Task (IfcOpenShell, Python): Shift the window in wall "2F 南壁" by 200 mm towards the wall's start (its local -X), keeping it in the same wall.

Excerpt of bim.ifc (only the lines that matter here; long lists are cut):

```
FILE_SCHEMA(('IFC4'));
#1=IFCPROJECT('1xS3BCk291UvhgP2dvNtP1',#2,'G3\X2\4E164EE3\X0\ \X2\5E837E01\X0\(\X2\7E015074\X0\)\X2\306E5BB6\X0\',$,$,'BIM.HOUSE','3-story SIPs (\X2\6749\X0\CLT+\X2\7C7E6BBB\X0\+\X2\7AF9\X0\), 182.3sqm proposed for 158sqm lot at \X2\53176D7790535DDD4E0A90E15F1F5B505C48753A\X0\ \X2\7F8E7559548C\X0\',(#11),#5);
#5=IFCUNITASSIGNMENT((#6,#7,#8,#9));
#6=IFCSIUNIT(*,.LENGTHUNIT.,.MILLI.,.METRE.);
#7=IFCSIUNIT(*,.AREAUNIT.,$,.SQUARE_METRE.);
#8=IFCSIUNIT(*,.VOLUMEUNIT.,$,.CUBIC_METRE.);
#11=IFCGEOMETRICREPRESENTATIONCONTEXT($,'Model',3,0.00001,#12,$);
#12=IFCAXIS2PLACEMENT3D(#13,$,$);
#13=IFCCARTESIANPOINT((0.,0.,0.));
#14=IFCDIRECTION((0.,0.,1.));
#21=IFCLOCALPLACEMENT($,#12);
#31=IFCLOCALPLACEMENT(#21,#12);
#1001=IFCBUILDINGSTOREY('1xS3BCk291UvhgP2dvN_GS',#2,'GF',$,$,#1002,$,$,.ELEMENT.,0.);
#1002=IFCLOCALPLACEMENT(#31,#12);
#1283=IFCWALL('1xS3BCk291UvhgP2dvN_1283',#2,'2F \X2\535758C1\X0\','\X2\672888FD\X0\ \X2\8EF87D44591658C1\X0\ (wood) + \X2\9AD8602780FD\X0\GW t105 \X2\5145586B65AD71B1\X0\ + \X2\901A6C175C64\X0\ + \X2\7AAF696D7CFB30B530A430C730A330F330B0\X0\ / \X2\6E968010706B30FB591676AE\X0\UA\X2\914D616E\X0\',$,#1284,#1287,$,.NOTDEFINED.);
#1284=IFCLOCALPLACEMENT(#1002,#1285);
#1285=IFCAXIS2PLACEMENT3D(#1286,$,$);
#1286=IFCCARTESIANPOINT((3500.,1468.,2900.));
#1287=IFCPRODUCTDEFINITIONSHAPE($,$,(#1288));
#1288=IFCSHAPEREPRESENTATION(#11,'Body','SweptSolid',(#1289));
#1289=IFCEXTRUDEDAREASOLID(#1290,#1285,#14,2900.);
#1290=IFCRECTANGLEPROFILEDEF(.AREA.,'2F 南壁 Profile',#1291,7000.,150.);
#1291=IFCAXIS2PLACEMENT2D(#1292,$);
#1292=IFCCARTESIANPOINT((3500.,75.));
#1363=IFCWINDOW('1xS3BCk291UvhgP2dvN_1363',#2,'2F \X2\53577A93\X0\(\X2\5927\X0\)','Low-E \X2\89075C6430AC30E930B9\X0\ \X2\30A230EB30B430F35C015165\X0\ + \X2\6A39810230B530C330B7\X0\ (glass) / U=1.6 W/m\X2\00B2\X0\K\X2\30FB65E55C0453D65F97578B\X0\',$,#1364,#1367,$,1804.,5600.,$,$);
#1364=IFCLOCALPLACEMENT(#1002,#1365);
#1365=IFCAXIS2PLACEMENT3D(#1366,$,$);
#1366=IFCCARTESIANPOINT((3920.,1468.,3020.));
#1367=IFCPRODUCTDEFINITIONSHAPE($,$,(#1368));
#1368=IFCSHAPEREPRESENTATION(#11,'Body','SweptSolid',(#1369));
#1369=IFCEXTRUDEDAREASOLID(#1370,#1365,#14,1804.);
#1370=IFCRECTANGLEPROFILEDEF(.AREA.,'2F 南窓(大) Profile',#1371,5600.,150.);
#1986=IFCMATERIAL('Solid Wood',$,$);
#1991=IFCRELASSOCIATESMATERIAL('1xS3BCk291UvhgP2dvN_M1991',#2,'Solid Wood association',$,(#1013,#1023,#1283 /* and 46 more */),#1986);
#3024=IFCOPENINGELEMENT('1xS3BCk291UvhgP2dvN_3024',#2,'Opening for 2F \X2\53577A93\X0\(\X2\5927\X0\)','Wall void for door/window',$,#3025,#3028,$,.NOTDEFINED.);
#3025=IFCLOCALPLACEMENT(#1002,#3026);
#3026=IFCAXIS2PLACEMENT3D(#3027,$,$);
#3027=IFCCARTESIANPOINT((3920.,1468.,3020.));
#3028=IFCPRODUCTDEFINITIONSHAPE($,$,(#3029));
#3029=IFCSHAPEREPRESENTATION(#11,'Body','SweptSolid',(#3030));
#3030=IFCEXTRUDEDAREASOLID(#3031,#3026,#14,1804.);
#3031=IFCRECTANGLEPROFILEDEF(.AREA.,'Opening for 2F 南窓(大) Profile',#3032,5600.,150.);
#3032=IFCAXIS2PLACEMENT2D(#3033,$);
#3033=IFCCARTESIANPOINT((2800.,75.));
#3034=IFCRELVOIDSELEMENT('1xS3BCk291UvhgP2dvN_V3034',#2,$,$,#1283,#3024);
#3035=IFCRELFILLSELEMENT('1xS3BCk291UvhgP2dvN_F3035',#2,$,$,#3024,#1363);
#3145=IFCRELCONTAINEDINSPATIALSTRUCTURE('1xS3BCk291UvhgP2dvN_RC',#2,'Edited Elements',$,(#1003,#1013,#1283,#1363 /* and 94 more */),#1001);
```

```python
import ifcopenshell
import ifcopenshell.api.geometry
import ifcopenshell.util.placement
import ifcopenshell.util.unit

model = ifcopenshell.open("bim.ifc")
unit_scale = ifcopenshell.util.unit.calculate_unit_scale(model)

window = model.by_guid("1xS3BCk291UvhgP2dvN_1363")
opening = window.FillsVoids[0].RelatingOpeningElement
wall = opening.VoidsElements[0].RelatingBuildingElement

wall_matrix = ifcopenshell.util.placement.get_local_placement(wall.ObjectPlacement)
shift = wall_matrix[:3, 0] * -0.2 / unit_scale
before = ifcopenshell.util.placement.get_local_placement(window.ObjectPlacement)[:3, 3].copy()

# The window is not placed relative to its opening, so move both.
for product in (opening, window):
    matrix = ifcopenshell.util.placement.get_local_placement(product.ObjectPlacement)
    matrix[:3, 3] += shift
    ifcopenshell.api.geometry.edit_object_placement(model, product=product, matrix=matrix, is_si=False)

after = ifcopenshell.util.placement.get_local_placement(window.ObjectPlacement)[:3, 3]
print("window moved by", (after - before).round(3) + 0.0)

model.write("bim-out.ifc")
```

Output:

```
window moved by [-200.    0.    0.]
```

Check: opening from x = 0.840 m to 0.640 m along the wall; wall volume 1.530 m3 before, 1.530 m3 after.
